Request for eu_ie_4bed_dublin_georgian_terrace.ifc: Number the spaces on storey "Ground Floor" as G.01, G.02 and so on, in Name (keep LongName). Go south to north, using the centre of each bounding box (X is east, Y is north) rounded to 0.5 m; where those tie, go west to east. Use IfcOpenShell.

First a look at what the model holds.

```python
import ifcopenshell
import ifcopenshell.util.element
import ifcopenshell.util.placement

model = ifcopenshell.open("eu_ie_4bed_dublin_georgian_terrace.ifc")
print(model.schema)
storey = next(s for s in model.by_type("IfcBuildingStorey") if s.Name == "Ground Floor")
spaces = [e for e in ifcopenshell.util.element.get_decomposition(storey) if e.is_a("IfcSpace")]
for e in sorted(spaces, key=lambda e: e.id()):
    origin = ifcopenshell.util.placement.get_local_placement(e.ObjectPlacement)[:3, 3]
    print(e.id(), e.Name, e.LongName, origin.round(2) + 0.0, sep=" | ")
```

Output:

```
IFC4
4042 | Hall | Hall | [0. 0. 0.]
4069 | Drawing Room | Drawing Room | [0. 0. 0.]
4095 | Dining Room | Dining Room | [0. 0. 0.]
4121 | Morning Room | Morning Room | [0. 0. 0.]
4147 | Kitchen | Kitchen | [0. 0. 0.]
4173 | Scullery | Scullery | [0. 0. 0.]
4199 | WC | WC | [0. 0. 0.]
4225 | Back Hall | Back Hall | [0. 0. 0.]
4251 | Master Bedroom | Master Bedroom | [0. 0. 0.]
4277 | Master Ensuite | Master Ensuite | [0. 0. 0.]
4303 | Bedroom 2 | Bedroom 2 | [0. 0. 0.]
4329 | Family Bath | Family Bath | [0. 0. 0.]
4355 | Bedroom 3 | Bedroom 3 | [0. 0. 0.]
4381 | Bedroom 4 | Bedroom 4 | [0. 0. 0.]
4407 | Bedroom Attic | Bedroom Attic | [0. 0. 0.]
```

```python
import ifcopenshell
import ifcopenshell.geom
import ifcopenshell.util.element
import ifcopenshell.util.shape

model = ifcopenshell.open("eu_ie_4bed_dublin_georgian_terrace.ifc")
settings = ifcopenshell.geom.settings()
settings.set("use-world-coords", True)


def centre(element):
    shape = ifcopenshell.geom.create_shape(settings, element)
    return ifcopenshell.util.shape.get_bbox_centroid(shape.geometry)


storey = next(s for s in model.by_type("IfcBuildingStorey") if s.Name == "Ground Floor")
spaces = [e for e in ifcopenshell.util.element.get_decomposition(storey) if e.is_a("IfcSpace")]

# Insertion points can sit at a corner or the storey origin, so sort by the geometry (in metres).
centres = {e: centre(e) for e in spaces}
spaces.sort(key=lambda e: (round(centres[e][1] / 0.5), centres[e][0]))

for i, e in enumerate(spaces, start=1):
    number = f"G.{i:02d}"
    e.Name = number
    print(e.id(), number)

model.write("eu_ie_4bed_dublin_georgian_terrace_rev.ifc")
```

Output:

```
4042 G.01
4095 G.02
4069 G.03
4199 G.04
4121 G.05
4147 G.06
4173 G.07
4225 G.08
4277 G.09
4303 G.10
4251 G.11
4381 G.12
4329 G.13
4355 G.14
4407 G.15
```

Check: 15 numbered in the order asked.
